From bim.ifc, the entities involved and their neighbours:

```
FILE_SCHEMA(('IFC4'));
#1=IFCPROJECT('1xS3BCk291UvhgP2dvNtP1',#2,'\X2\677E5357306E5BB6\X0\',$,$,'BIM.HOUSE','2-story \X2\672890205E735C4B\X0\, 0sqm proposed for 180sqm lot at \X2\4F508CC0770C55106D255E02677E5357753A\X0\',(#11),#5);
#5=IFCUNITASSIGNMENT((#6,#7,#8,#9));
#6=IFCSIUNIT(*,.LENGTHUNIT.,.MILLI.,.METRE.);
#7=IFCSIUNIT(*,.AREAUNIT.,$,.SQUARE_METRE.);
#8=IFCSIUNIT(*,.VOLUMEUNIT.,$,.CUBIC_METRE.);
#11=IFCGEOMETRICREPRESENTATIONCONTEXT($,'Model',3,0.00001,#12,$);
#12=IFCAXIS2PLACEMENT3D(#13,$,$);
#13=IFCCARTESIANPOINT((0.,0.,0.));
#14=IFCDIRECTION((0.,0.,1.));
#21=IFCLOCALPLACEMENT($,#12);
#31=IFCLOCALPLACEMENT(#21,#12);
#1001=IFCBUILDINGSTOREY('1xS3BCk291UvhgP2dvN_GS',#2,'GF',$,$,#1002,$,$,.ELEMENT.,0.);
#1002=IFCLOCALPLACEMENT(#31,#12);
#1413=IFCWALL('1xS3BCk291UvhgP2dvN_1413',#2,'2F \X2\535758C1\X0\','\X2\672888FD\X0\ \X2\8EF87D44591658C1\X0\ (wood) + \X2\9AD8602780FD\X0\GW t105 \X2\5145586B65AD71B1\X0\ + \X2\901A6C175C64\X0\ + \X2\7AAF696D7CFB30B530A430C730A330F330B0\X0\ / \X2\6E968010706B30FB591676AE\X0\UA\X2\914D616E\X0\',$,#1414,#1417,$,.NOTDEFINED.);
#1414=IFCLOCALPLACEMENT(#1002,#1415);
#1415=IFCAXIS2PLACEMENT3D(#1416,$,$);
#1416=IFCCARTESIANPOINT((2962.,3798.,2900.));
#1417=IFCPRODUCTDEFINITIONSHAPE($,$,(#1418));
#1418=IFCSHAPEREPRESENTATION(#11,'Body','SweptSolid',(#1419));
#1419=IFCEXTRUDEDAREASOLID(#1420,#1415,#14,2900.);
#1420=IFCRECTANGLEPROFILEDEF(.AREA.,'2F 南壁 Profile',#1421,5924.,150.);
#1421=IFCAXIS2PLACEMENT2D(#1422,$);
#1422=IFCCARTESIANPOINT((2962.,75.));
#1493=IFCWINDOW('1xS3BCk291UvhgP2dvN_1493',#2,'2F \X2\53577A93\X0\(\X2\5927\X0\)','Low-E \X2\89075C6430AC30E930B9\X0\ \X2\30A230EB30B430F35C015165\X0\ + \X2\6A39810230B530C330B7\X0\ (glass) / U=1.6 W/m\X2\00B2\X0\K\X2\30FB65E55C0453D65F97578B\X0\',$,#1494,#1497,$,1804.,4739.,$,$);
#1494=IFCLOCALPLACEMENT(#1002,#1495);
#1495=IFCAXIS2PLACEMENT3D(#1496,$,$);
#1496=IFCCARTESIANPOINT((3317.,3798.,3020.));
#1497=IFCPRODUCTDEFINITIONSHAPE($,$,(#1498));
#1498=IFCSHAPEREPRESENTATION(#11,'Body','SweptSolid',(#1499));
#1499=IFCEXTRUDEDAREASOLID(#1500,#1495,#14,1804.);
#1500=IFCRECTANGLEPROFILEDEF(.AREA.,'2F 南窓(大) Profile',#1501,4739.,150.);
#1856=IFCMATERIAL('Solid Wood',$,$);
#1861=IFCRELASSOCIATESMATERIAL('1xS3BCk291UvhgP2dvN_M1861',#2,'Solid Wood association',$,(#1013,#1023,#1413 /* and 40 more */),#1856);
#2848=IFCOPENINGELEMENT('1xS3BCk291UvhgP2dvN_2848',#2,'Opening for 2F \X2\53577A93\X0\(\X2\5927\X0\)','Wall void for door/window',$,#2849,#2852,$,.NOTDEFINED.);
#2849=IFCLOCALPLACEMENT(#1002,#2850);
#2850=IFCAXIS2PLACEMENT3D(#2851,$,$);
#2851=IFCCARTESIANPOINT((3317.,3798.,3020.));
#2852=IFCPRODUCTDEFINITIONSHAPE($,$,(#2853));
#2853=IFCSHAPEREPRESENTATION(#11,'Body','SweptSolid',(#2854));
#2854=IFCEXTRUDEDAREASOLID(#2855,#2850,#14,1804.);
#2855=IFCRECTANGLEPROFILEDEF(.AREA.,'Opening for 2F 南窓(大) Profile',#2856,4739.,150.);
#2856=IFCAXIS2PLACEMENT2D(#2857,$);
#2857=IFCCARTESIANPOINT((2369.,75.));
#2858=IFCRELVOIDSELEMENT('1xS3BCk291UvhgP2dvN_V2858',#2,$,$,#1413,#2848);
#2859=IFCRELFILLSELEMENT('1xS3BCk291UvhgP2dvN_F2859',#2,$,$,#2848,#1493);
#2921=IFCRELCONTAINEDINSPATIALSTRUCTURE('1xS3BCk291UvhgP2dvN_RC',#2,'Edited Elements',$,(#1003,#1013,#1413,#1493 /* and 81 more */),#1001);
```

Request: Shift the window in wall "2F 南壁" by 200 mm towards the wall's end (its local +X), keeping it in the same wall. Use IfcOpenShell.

```python
import ifcopenshell
import ifcopenshell.api.geometry
import ifcopenshell.util.placement
import ifcopenshell.util.unit

model = ifcopenshell.open("bim.ifc")
unit_scale = ifcopenshell.util.unit.calculate_unit_scale(model)

window = model.by_guid("1xS3BCk291UvhgP2dvN_1493")
opening = window.FillsVoids[0].RelatingOpeningElement
wall = opening.VoidsElements[0].RelatingBuildingElement

wall_matrix = ifcopenshell.util.placement.get_local_placement(wall.ObjectPlacement)
shift = wall_matrix[:3, 0] * 0.2 / unit_scale
before = ifcopenshell.util.placement.get_local_placement(window.ObjectPlacement)[:3, 3].copy()

# The window is not placed relative to its opening, so move both.
for product in (opening, window):
    matrix = ifcopenshell.util.placement.get_local_placement(product.ObjectPlacement)
    matrix[:3, 3] += shift
    ifcopenshell.api.geometry.edit_object_placement(model, product=product, matrix=matrix, is_si=False)

after = ifcopenshell.util.placement.get_local_placement(window.ObjectPlacement)[:3, 3]
print("window moved by", (after - before).round(3) + 0.0)

model.write("bim_updated.ifc")
```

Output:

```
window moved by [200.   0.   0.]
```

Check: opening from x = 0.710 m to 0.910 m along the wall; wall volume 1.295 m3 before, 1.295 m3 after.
